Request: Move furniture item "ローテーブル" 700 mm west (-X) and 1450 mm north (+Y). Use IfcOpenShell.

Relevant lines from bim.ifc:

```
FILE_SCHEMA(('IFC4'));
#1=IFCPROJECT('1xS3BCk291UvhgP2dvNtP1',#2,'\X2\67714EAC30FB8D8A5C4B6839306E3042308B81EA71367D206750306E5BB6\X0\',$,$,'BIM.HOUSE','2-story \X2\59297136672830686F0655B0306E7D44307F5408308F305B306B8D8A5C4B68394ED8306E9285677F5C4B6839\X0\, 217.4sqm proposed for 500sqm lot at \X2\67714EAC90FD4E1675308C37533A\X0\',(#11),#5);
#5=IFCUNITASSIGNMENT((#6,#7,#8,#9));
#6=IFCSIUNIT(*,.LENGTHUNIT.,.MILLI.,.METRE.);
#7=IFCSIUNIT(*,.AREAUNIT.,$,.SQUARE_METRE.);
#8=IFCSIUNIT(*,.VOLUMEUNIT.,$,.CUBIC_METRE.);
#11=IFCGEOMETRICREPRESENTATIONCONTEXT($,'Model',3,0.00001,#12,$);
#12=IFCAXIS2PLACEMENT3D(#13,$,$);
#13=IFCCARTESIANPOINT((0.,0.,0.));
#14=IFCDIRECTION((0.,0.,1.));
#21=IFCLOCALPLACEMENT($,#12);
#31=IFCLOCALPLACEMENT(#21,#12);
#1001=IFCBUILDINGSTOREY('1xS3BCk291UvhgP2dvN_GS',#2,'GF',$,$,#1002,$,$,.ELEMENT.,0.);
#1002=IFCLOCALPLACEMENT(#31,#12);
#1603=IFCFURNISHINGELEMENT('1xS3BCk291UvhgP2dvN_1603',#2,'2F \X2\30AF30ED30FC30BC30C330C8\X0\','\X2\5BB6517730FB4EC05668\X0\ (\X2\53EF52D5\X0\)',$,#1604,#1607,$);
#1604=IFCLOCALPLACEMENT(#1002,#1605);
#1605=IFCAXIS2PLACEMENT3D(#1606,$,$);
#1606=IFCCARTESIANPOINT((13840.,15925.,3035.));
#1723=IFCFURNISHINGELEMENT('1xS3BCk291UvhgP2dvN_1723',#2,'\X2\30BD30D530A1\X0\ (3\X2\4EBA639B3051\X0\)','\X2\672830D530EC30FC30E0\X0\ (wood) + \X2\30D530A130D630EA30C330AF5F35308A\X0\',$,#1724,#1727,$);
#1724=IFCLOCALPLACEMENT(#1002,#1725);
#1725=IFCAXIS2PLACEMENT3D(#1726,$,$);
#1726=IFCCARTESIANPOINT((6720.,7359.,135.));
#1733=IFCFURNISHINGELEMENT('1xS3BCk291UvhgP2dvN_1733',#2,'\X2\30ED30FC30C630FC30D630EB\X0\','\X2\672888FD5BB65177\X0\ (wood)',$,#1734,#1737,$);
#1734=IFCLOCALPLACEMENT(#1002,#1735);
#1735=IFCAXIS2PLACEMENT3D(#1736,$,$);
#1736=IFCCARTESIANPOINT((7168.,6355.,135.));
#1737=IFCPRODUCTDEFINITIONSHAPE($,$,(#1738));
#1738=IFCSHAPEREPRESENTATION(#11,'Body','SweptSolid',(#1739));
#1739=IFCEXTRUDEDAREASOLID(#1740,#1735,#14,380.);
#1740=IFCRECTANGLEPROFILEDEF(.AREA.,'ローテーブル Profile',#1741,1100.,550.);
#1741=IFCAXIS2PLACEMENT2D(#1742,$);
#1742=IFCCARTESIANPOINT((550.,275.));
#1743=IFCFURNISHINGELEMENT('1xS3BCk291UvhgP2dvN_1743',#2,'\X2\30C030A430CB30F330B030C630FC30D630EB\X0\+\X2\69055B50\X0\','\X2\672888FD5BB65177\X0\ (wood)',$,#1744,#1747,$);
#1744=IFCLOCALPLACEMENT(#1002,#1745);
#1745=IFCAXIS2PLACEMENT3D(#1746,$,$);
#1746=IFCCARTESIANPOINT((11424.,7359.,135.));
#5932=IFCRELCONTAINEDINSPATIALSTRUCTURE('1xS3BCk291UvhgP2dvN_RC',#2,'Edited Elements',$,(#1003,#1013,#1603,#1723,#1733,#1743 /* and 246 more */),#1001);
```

```python
import ifcopenshell
import ifcopenshell.api.geometry
import ifcopenshell.util.placement

model = ifcopenshell.open("bim.ifc")

item = model.by_id(1733)
matrix = ifcopenshell.util.placement.get_local_placement(item.ObjectPlacement)
matrix[0, 3] -= 700.0
matrix[1, 3] += 1450.0
ifcopenshell.api.geometry.edit_object_placement(model, product=item, matrix=matrix, is_si=False)

print(ifcopenshell.util.placement.get_local_placement(item.ObjectPlacement).round(3) + 0.0)

model.write("bim_updated.ifc")
```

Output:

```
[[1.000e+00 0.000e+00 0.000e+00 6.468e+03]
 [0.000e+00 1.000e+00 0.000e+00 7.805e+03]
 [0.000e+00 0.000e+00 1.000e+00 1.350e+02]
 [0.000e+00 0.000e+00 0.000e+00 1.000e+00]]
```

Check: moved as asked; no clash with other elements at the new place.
